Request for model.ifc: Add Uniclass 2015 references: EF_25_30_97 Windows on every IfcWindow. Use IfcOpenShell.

First a look at what the model holds.

```python
import ifcopenshell

model = ifcopenshell.open("model.ifc")
print(model.schema)
print("classifications:", [c.Name for c in model.by_type("IfcClassification")])
for ifc_class in ("IfcDoor", "IfcRoof", "IfcStair", "IfcWall", "IfcWindow"):
    print(ifc_class, len(model.by_type(ifc_class)))
```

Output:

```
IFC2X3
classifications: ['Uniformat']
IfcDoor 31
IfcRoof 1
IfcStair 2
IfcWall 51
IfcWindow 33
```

```python
import ifcopenshell
import ifcopenshell.api.classification

model = ifcopenshell.open("model.ifc")

# IFC2X3 requires Source and Edition and has no link from the project to the system.
system = model.create_entity("IfcClassification", Source="NBS", Edition="2015", Name="Uniclass 2015")

codes = {
    "IfcWindow": ("EF_25_30_97", "Windows"),
}
for ifc_class, (code, name) in codes.items():
    products = model.by_type(ifc_class)
    ifcopenshell.api.classification.add_reference(
        model, products=products, classification=system, identification=code, name=name
    )
    print(code, len(products))

model.write("model_edited.ifc")
```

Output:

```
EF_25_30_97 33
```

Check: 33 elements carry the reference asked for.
